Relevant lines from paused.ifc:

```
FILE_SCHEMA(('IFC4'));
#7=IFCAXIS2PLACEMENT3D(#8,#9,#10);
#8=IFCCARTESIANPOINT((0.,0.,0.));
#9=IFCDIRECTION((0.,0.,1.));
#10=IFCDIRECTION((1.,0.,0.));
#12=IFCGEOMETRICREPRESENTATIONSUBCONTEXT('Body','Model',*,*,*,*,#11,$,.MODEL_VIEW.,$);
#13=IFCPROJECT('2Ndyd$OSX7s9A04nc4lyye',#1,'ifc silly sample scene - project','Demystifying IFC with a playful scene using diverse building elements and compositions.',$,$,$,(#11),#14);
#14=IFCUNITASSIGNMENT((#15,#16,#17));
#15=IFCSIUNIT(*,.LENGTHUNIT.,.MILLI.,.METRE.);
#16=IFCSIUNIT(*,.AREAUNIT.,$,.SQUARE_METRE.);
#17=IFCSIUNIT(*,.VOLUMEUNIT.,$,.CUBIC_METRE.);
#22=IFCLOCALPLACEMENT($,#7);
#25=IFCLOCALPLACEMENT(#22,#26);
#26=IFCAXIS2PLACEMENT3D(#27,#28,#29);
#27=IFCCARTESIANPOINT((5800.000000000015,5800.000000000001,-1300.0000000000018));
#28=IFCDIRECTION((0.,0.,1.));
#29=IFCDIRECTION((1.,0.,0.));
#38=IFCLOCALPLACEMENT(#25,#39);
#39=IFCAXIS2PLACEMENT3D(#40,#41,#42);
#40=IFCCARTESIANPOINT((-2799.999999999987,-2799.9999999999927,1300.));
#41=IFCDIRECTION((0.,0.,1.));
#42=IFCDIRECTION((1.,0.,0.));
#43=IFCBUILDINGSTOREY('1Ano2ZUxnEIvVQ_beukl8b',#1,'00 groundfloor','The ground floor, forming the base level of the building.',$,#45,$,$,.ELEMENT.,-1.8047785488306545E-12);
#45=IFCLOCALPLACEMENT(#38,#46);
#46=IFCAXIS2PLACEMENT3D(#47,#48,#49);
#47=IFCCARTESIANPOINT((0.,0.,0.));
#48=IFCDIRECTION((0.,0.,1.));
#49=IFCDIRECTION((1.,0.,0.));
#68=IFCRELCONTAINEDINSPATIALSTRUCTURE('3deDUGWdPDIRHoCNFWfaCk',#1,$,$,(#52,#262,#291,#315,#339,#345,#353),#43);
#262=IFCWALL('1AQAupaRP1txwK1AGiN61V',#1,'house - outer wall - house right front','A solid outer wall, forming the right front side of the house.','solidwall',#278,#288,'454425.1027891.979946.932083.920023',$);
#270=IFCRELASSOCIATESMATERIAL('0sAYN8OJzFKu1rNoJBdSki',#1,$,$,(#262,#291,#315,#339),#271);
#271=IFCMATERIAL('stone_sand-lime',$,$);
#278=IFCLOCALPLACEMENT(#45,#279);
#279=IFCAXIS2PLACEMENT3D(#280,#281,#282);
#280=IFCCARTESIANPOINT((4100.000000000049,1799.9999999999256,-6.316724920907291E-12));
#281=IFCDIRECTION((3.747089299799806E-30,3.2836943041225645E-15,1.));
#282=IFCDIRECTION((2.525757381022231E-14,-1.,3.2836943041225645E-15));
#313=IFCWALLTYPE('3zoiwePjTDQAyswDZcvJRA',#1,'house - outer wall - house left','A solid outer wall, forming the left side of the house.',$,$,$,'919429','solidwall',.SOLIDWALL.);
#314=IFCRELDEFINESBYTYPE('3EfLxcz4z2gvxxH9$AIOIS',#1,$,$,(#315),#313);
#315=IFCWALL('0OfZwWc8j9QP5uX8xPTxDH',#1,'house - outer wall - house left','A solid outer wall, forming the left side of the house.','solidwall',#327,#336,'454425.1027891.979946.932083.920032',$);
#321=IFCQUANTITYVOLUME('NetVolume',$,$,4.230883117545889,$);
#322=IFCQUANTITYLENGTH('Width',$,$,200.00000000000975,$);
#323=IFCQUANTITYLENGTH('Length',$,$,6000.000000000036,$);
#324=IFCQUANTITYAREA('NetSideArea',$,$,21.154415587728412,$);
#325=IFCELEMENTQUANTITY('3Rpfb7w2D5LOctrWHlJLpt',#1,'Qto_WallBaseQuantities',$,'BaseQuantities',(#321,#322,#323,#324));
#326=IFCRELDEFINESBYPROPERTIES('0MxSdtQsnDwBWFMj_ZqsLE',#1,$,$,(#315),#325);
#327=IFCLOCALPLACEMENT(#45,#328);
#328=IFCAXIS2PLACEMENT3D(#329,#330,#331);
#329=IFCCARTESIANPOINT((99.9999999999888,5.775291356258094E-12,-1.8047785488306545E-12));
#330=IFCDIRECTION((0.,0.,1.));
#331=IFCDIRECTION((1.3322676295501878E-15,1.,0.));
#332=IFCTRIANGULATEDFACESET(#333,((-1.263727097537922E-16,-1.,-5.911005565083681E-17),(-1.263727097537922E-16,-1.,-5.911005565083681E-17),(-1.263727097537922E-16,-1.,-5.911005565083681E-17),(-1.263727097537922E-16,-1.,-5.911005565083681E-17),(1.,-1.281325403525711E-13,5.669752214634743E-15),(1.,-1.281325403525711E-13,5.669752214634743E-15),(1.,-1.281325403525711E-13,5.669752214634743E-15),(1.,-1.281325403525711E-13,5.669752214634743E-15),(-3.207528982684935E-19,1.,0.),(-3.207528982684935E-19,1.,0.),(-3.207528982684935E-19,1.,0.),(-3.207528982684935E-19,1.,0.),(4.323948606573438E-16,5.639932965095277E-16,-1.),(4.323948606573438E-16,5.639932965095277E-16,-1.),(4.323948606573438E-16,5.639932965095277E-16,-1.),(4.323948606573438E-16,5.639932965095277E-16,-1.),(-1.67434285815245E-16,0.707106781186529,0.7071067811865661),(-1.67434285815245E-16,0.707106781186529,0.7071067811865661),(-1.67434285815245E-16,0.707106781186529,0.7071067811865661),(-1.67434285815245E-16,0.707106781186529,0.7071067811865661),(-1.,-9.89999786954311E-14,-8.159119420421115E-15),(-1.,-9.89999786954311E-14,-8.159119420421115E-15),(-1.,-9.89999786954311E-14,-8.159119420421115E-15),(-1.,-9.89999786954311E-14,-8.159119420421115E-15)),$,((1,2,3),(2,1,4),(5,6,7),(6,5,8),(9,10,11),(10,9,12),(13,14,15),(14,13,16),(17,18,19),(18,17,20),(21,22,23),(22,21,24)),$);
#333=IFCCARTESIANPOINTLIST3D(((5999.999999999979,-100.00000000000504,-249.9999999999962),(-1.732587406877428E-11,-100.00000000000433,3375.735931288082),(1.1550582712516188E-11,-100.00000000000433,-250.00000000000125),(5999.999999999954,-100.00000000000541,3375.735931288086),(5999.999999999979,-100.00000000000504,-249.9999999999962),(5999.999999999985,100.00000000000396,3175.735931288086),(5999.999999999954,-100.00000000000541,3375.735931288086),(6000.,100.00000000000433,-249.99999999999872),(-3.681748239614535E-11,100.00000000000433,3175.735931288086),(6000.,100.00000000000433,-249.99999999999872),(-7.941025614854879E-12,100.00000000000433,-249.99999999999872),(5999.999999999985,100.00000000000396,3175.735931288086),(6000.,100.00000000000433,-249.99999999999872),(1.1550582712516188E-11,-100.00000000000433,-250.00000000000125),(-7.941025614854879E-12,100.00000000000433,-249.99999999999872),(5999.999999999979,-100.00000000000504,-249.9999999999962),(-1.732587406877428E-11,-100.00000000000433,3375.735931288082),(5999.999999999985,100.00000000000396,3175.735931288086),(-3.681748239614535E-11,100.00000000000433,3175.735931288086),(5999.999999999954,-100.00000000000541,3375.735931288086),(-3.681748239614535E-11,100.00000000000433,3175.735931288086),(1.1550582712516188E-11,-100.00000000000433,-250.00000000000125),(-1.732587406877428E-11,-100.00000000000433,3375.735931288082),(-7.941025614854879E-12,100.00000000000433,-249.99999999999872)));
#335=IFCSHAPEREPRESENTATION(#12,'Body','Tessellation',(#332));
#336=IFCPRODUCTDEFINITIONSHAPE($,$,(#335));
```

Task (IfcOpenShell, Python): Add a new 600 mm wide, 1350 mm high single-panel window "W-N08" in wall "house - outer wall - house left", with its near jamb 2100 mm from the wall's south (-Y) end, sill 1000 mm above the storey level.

```python
import numpy as np
import ifcopenshell
import ifcopenshell.api.feature
import ifcopenshell.api.geometry
import ifcopenshell.api.pset
import ifcopenshell.api.root
import ifcopenshell.api.spatial
import ifcopenshell.geom
import ifcopenshell.util.element
import ifcopenshell.util.placement
import ifcopenshell.util.representation
import ifcopenshell.util.shape
import ifcopenshell.util.unit

model = ifcopenshell.open("paused.ifc")
unit_scale = ifcopenshell.util.unit.calculate_unit_scale(model)
area_scale = ifcopenshell.util.unit.calculate_unit_scale(model, "AREAUNIT")
volume_scale = ifcopenshell.util.unit.calculate_unit_scale(model, "VOLUMEUNIT")
settings = ifcopenshell.geom.settings()


def volume(element):
    """Net volume in cubic metres, openings subtracted."""
    shape = ifcopenshell.geom.create_shape(settings, element)
    return ifcopenshell.util.shape.get_volume(shape.geometry)


wall = model.by_guid("0OfZwWc8j9QP5uX8xPTxDH")
storey = ifcopenshell.util.element.get_container(wall, ifc_class="IfcBuildingStorey")
context = ifcopenshell.util.representation.get_context(model, "Model", "Body", "MODEL_VIEW")
before = volume(wall)

width, height, from_end, sill = 0.6, 1.35, 2.1, 1  # metres

# The wall runs along its own X axis, and the end named is its -X end.
wall_shape = ifcopenshell.geom.create_shape(settings, wall)
x, y, z = ifcopenshell.util.shape.get_vertices(wall_shape.geometry).T
start = x.min() + from_end
face, thickness = float(y.min()), float(y.max() - y.min())
wall_matrix = ifcopenshell.util.placement.get_local_placement(wall.ObjectPlacement)
level = ifcopenshell.util.placement.get_local_placement(storey.ObjectPlacement)[2, 3]


def in_wall(x, y):
    """Placement at x, y metres in the wall's axes, at sill height."""
    matrix = wall_matrix.copy()
    matrix[:, 3] = wall_matrix @ np.array([x / unit_scale, y / unit_scale, 0.0, 1.0])
    matrix[2, 3] = level + sill / unit_scale
    return matrix


# Opening: a box that overshoots both wall faces by 50 mm.
opening = ifcopenshell.api.root.create_entity(model, ifc_class="IfcOpeningElement", predefined_type="OPENING")
box = ifcopenshell.api.geometry.add_wall_representation(
    model, context=context, length=width, height=height, thickness=thickness + 0.1
)
ifcopenshell.api.geometry.assign_representation(model, product=opening, representation=box)
ifcopenshell.api.geometry.edit_object_placement(model, product=opening, matrix=in_wall(start, face - 0.05), is_si=False)
ifcopenshell.api.feature.add_feature(model, feature=opening, element=wall)

window = ifcopenshell.api.root.create_entity(model, ifc_class="IfcWindow", name="W-N08", predefined_type="WINDOW")
window.OverallWidth, window.OverallHeight = width / unit_scale, height / unit_scale
window.PartitioningType = "SINGLE_PANEL"
body = ifcopenshell.api.geometry.add_window_representation(
    model,
    context=context,
    overall_width=window.OverallWidth,
    overall_height=window.OverallHeight,
    partition_type="SINGLE_PANEL",
)
ifcopenshell.api.geometry.assign_representation(model, product=window, representation=body)
ifcopenshell.api.spatial.assign_container(model, products=[window], relating_structure=storey)
ifcopenshell.api.feature.add_filling(model, opening=opening, element=window)

# Centre the window in the wall's thickness.
ifcopenshell.api.geometry.edit_object_placement(model, product=window, matrix=in_wall(start, face), is_si=False)
window_shape = ifcopenshell.geom.create_shape(settings, window)
depth = ifcopenshell.util.shape.get_vertices(window_shape.geometry)[:, 1]
offset = face + thickness / 2 - (depth.min() + depth.max()) / 2
ifcopenshell.api.geometry.edit_object_placement(model, product=window, matrix=in_wall(start, offset), is_si=False)

after = volume(wall)

# Update the wall's stored quantities.
qto = model.by_id(ifcopenshell.util.element.get_pset(wall, "Qto_WallBaseQuantities", should_inherit=False)["id"])
ifcopenshell.api.pset.edit_qto(model, qto=qto, properties={
    "NetVolume": after / volume_scale,
    "NetSideArea": after / thickness / area_scale,
})

print(f"wall volume {before:.3f} -> {after:.3f} m3")

model.write("paused_updated.ifc")
```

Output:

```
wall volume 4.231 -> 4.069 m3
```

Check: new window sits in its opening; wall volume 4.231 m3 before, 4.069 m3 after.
